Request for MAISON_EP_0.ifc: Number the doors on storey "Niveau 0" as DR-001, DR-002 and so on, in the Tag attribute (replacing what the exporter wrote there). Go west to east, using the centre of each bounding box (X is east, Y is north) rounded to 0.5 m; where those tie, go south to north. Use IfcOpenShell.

First a look at what the model holds.

```python
import ifcopenshell
import ifcopenshell.util.element
import ifcopenshell.util.placement

model = ifcopenshell.open("MAISON_EP_0.ifc")
print(model.schema)
storey = next(s for s in model.by_type("IfcBuildingStorey") if s.Name == "Niveau 0")
doors = [e for e in ifcopenshell.util.element.get_decomposition(storey) if e.is_a("IfcDoor")]
for e in sorted(doors, key=lambda e: e.id()):
    origin = ifcopenshell.util.placement.get_local_placement(e.ObjectPlacement)[:3, 3]
    print(e.id(), e.Tag, e.Name, origin.round(2) + 0.0, sep=" | ")
```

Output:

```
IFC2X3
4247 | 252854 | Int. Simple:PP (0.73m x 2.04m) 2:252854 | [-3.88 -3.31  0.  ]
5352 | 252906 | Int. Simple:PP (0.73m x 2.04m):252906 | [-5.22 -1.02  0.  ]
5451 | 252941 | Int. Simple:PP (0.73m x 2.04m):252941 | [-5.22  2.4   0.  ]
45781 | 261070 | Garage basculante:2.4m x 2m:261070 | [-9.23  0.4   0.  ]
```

```python
import ifcopenshell
import ifcopenshell.geom
import ifcopenshell.util.element
import ifcopenshell.util.shape

model = ifcopenshell.open("MAISON_EP_0.ifc")
settings = ifcopenshell.geom.settings()
settings.set("use-world-coords", True)


def centre(element):
    shape = ifcopenshell.geom.create_shape(settings, element)
    return ifcopenshell.util.shape.get_bbox_centroid(shape.geometry)


storey = next(s for s in model.by_type("IfcBuildingStorey") if s.Name == "Niveau 0")
doors = [e for e in ifcopenshell.util.element.get_decomposition(storey) if e.is_a("IfcDoor")]

# Insertion points can sit at a corner or the storey origin, so sort by the geometry (in metres).
centres = {e: centre(e) for e in doors}
doors.sort(key=lambda e: (round(centres[e][0] / 0.5), centres[e][1]))

for i, e in enumerate(doors, start=1):
    number = f"DR-0{i:02d}"
    e.Tag = number
    print(e.id(), number)

model.write("MAISON_EP_0_updated.ifc")
```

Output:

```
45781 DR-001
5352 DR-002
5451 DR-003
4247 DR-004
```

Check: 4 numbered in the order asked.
